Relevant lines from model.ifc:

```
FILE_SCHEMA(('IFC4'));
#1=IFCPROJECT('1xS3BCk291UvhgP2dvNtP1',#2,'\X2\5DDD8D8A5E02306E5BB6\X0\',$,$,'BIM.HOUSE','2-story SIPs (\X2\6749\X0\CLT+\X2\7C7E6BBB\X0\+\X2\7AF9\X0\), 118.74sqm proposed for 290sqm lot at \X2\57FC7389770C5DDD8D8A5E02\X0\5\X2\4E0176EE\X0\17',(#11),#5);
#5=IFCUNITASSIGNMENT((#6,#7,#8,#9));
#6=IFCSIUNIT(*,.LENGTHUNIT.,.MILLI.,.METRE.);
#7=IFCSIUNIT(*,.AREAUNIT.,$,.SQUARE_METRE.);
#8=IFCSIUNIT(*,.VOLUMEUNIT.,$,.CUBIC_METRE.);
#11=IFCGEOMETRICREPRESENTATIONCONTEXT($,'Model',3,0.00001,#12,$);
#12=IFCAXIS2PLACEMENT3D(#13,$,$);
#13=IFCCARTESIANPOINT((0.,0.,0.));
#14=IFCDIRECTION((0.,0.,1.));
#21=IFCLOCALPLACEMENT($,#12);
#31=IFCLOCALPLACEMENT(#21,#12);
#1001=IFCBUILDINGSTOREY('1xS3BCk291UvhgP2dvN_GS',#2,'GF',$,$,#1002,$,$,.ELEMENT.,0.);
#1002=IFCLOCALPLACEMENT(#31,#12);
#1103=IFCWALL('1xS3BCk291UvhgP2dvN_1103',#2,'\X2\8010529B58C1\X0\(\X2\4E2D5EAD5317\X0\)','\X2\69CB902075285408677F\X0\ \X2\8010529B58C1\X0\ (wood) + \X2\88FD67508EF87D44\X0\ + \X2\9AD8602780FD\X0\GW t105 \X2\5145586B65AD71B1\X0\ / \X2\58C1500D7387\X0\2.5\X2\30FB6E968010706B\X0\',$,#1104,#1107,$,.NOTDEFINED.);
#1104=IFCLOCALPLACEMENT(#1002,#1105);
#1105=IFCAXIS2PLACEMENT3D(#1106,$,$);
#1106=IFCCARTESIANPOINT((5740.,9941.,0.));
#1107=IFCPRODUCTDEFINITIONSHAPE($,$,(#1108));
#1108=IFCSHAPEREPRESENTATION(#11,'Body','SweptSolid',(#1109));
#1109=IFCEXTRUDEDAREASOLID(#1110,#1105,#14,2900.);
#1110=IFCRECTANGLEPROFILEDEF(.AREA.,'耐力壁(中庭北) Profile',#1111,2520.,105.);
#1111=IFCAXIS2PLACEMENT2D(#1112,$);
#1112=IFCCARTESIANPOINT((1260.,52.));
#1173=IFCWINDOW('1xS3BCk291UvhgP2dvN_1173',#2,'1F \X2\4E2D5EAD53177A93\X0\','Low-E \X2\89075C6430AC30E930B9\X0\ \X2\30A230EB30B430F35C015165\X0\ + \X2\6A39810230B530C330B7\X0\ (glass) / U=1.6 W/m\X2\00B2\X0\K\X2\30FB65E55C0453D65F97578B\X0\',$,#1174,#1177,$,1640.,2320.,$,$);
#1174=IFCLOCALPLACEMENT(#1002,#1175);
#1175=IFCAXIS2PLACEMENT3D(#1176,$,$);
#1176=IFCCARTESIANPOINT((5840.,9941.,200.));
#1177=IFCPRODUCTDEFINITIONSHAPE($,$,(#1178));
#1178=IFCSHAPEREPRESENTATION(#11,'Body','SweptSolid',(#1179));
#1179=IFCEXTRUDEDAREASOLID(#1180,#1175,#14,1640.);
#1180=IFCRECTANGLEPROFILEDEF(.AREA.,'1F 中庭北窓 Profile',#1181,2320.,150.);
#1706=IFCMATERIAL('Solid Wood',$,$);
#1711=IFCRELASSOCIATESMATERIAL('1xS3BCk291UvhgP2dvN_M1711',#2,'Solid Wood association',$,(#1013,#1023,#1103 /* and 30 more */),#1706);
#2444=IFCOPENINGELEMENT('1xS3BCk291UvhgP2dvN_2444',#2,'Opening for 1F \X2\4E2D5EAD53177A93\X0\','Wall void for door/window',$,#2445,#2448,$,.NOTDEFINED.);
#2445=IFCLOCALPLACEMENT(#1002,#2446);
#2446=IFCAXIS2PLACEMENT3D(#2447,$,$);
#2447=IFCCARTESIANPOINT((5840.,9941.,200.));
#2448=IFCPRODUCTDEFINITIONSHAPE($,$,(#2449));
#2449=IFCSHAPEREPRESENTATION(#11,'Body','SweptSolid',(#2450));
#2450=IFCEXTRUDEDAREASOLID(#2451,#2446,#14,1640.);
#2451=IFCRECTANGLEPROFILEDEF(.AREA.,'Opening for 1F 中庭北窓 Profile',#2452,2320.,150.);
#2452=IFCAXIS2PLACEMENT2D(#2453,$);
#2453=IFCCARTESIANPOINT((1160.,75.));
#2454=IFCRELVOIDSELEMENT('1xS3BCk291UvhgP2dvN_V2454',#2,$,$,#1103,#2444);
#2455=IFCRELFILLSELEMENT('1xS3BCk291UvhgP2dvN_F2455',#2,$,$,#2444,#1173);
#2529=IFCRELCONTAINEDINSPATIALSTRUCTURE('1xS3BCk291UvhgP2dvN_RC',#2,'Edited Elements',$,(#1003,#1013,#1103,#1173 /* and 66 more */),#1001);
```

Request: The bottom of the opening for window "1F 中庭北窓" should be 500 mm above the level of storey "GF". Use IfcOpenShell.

```python
import numpy as np
import ifcopenshell
import ifcopenshell.api.geometry
import ifcopenshell.geom
import ifcopenshell.util.element
import ifcopenshell.util.placement
import ifcopenshell.util.shape
import ifcopenshell.util.unit

model = ifcopenshell.open("model.ifc")
unit_scale = ifcopenshell.util.unit.calculate_unit_scale(model)

window = model.by_guid("1xS3BCk291UvhgP2dvN_1173")
opening = window.FillsVoids[0].RelatingOpeningElement
storey = ifcopenshell.util.element.get_container(window, ifc_class="IfcBuildingStorey")
level = ifcopenshell.util.placement.get_local_placement(storey.ObjectPlacement)[2, 3]

# The opening's origin need not be at the sill, so measure its lowest point.
shape = ifcopenshell.geom.create_shape(ifcopenshell.geom.settings(), opening)
bottom = ifcopenshell.util.shape.get_shape_bottom_elevation(shape, shape.geometry) / unit_scale
dz = level + 0.5 / unit_scale - bottom

shift = np.array([0.0, 0.0, dz])
# The window is not placed relative to its opening, so move both.
for product in (opening, window):
    matrix = ifcopenshell.util.placement.get_local_placement(product.ObjectPlacement)
    matrix[:3, 3] += shift
    ifcopenshell.api.geometry.edit_object_placement(model, product=product, matrix=matrix, is_si=False)

print(f"moved by {dz * unit_scale:+.3f} m")

model.write("model_updated.ifc")
```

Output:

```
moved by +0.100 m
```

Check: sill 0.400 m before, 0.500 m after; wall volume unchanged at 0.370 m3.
